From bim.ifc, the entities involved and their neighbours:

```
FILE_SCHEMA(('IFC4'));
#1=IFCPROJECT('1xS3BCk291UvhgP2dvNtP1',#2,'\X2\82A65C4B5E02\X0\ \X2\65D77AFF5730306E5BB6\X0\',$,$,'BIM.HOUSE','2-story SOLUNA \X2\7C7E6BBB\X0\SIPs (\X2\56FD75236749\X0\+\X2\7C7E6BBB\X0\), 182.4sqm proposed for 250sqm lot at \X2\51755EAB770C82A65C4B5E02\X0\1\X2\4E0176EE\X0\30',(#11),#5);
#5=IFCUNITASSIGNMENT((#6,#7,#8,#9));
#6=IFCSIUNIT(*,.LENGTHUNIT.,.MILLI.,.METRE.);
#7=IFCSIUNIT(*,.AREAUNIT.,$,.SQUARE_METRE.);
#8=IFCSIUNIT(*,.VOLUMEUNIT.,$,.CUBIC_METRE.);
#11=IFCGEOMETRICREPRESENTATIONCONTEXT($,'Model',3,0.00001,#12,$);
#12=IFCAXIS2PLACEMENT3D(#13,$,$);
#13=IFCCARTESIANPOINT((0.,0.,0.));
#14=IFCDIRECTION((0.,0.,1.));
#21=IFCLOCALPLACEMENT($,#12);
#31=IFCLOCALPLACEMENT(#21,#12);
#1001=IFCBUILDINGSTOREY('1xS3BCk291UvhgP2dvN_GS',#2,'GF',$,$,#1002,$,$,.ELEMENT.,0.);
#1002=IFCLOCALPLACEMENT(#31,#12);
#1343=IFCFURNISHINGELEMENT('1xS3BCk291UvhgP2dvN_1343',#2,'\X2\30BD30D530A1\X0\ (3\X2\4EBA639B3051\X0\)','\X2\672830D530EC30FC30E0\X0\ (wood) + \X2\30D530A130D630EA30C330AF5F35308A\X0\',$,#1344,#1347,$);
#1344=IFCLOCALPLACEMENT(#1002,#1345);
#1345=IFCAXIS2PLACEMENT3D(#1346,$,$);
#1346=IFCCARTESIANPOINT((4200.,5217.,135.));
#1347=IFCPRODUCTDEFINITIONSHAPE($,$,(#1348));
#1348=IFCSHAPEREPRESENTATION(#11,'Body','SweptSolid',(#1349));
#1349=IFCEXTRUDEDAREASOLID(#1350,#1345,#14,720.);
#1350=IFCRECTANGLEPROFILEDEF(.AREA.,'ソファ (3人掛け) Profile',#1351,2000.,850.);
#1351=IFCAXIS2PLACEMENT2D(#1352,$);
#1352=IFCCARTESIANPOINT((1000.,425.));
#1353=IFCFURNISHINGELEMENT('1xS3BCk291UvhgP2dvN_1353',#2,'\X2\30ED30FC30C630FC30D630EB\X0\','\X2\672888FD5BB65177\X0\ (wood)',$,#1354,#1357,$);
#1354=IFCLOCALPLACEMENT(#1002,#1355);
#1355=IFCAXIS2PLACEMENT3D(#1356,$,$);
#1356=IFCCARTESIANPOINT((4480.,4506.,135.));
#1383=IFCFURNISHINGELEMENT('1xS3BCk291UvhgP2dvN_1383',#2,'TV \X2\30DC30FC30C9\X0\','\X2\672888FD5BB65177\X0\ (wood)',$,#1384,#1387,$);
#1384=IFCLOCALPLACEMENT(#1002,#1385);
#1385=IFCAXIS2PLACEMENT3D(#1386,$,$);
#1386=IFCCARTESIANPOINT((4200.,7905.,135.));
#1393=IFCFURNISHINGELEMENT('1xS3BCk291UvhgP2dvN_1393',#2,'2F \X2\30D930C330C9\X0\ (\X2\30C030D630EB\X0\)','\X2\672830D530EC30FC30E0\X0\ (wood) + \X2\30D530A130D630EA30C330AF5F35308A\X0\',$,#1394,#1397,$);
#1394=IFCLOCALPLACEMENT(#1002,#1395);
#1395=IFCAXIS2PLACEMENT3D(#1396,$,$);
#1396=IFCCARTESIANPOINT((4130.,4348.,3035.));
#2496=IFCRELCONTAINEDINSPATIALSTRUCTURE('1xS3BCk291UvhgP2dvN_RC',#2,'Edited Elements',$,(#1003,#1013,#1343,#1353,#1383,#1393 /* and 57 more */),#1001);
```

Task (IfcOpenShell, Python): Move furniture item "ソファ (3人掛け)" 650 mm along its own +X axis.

```python
import ifcopenshell
import ifcopenshell.api.geometry
import ifcopenshell.util.placement
import ifcopenshell.util.unit

model = ifcopenshell.open("bim.ifc")
unit_scale = ifcopenshell.util.unit.calculate_unit_scale(model)

item = model.by_guid("1xS3BCk291UvhgP2dvN_1343")
matrix = ifcopenshell.util.placement.get_local_placement(item.ObjectPlacement)
matrix[:3, 3] += matrix[:3, 0] * 0.65 / unit_scale
ifcopenshell.api.geometry.edit_object_placement(model, product=item, matrix=matrix, is_si=False)

print(ifcopenshell.util.placement.get_local_placement(item.ObjectPlacement).round(3) + 0.0)

model.write("bim_edited.ifc")
```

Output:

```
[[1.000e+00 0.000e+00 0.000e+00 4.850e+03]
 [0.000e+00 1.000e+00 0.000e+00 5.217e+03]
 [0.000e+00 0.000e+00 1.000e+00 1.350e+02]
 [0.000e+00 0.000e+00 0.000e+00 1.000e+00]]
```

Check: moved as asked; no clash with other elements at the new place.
